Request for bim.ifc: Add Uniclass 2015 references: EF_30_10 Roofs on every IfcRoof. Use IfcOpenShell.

First a look at what the model holds.

```python
import ifcopenshell

model = ifcopenshell.open("bim.ifc")
print(model.schema)
print("classifications:", [c.Name for c in model.by_type("IfcClassification")])
for ifc_class in ("IfcDoor", "IfcRoof", "IfcStair", "IfcWall", "IfcWindow"):
    print(ifc_class, len(model.by_type(ifc_class)))
```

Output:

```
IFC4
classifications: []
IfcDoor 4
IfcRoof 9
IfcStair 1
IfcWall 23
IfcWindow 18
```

```python
import ifcopenshell
import ifcopenshell.api.classification

model = ifcopenshell.open("bim.ifc")

system = ifcopenshell.api.classification.add_classification(model, classification="Uniclass 2015")

codes = {
    "IfcRoof": ("EF_30_10", "Roofs"),
}
for ifc_class, (code, name) in codes.items():
    products = model.by_type(ifc_class)
    ifcopenshell.api.classification.add_reference(
        model, products=products, classification=system, identification=code, name=name
    )
    print(code, len(products))

model.write("bim_v2.ifc")
```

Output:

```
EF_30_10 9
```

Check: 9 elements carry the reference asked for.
